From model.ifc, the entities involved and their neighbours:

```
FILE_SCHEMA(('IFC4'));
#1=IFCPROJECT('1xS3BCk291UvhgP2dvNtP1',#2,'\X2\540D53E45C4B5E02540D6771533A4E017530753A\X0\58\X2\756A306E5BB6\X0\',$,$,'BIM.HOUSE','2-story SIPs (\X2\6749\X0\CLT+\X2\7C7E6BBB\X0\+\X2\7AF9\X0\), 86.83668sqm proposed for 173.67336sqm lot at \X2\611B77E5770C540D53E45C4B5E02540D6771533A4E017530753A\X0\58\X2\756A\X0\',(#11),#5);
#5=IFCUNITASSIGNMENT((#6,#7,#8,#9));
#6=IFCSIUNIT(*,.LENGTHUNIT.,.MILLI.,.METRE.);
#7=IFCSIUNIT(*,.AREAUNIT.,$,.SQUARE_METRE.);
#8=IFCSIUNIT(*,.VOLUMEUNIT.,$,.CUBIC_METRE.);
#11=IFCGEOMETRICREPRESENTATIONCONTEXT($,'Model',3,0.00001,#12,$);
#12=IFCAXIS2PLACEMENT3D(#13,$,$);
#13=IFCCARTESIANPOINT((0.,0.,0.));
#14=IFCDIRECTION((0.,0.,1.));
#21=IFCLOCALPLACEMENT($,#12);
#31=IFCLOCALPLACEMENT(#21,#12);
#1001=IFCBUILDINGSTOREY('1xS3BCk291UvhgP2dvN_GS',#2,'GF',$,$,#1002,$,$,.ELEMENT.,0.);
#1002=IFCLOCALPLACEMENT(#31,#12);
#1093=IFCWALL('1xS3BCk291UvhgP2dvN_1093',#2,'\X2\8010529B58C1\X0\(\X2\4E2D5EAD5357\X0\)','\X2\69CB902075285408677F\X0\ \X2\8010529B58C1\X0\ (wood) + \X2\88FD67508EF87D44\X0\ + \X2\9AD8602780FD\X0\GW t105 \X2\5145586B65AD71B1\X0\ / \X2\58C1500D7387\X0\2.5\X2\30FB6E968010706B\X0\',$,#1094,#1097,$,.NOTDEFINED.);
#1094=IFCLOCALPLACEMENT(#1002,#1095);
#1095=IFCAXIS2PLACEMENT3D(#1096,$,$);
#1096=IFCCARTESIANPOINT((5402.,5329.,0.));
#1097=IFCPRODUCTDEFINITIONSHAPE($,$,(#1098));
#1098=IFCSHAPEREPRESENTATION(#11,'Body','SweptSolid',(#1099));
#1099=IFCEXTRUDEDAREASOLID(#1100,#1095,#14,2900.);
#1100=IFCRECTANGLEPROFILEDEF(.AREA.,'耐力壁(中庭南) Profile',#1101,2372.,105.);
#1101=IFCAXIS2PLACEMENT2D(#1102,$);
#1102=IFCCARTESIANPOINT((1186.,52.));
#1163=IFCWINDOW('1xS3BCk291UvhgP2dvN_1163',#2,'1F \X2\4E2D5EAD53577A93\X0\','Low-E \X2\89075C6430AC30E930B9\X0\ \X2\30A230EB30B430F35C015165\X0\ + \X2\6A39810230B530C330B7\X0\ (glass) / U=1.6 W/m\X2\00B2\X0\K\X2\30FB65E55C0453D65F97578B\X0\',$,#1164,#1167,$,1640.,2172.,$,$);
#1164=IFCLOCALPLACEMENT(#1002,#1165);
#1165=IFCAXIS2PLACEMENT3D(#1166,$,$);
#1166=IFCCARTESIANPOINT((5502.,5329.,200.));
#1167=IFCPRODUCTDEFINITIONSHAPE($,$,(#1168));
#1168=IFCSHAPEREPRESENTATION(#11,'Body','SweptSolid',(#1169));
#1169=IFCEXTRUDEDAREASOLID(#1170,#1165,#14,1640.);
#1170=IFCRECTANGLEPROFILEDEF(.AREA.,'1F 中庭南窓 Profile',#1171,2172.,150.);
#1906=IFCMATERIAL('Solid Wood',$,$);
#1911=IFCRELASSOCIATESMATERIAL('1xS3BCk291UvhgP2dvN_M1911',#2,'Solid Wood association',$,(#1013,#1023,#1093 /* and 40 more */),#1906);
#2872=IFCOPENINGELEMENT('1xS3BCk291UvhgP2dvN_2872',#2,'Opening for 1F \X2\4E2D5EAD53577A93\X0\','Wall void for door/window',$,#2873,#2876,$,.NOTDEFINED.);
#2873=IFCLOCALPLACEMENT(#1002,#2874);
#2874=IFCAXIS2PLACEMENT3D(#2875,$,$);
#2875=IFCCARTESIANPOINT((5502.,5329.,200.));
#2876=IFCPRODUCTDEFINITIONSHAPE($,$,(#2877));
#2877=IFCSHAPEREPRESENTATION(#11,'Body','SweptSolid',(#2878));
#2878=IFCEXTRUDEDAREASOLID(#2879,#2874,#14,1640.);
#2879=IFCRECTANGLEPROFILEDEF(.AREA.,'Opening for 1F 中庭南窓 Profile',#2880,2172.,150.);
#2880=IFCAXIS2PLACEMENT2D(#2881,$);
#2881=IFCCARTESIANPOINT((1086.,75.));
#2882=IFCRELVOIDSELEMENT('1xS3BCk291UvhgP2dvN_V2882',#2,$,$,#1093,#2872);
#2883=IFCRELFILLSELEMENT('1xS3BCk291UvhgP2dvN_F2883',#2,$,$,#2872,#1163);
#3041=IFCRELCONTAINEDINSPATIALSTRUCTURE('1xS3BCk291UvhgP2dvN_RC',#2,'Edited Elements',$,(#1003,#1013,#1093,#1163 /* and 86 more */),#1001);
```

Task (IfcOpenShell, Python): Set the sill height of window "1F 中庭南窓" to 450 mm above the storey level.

```python
import numpy as np
import ifcopenshell
import ifcopenshell.api.geometry
import ifcopenshell.geom
import ifcopenshell.util.element
import ifcopenshell.util.placement
import ifcopenshell.util.shape
import ifcopenshell.util.unit

model = ifcopenshell.open("model.ifc")
unit_scale = ifcopenshell.util.unit.calculate_unit_scale(model)

window = model.by_id(1163)
opening = window.FillsVoids[0].RelatingOpeningElement
storey = ifcopenshell.util.element.get_container(window, ifc_class="IfcBuildingStorey")
level = ifcopenshell.util.placement.get_local_placement(storey.ObjectPlacement)[2, 3]

# The opening's origin need not be at the sill, so measure its lowest point.
shape = ifcopenshell.geom.create_shape(ifcopenshell.geom.settings(), opening)
bottom = ifcopenshell.util.shape.get_shape_bottom_elevation(shape, shape.geometry) / unit_scale
dz = level + 0.45 / unit_scale - bottom

shift = np.array([0.0, 0.0, dz])
# The window is not placed relative to its opening, so move both.
for product in (opening, window):
    matrix = ifcopenshell.util.placement.get_local_placement(product.ObjectPlacement)
    matrix[:3, 3] += shift
    ifcopenshell.api.geometry.edit_object_placement(model, product=product, matrix=matrix, is_si=False)

print(f"moved by {dz * unit_scale:+.3f} m")

model.write("model-out.ifc")
```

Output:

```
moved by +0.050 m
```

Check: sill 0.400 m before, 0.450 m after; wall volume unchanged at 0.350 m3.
